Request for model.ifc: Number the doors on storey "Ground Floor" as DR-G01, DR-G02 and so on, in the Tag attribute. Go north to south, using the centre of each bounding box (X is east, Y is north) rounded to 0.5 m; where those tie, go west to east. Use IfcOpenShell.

First a look at what the model holds.

```python
import ifcopenshell
import ifcopenshell.util.element
import ifcopenshell.util.placement

model = ifcopenshell.open("model.ifc")
print(model.schema)
storey = next(s for s in model.by_type("IfcBuildingStorey") if s.Name == "Ground Floor")
doors = [e for e in ifcopenshell.util.element.get_decomposition(storey) if e.is_a("IfcDoor")]
for e in sorted(doors, key=lambda e: e.id()):
    origin = ifcopenshell.util.placement.get_local_placement(e.ObjectPlacement)[:3, 3]
    print(e.id(), e.Tag, e.Name, origin.round(2) + 0.0, sep=" | ")
```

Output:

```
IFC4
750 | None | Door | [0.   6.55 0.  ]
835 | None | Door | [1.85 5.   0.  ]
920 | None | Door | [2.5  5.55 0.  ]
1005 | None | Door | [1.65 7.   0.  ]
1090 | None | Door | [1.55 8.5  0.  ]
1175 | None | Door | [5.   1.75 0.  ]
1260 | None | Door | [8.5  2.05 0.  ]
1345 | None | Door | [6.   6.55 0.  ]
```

```python
import ifcopenshell
import ifcopenshell.geom
import ifcopenshell.util.element
import ifcopenshell.util.shape

model = ifcopenshell.open("model.ifc")
settings = ifcopenshell.geom.settings()
settings.set("use-world-coords", True)


def centre(element):
    shape = ifcopenshell.geom.create_shape(settings, element)
    return ifcopenshell.util.shape.get_bbox_centroid(shape.geometry)


storey = next(s for s in model.by_type("IfcBuildingStorey") if s.Name == "Ground Floor")
doors = [e for e in ifcopenshell.util.element.get_decomposition(storey) if e.is_a("IfcDoor")]

# Insertion points can sit at a corner or the storey origin, so sort by the geometry (in metres).
centres = {e: centre(e) for e in doors}
doors.sort(key=lambda e: (-round(centres[e][1] / 0.5), centres[e][0]))

for i, e in enumerate(doors, start=1):
    number = f"DR-G{i:02d}"
    e.Tag = number
    print(e.id(), number)

model.write("model_edited.ifc")
```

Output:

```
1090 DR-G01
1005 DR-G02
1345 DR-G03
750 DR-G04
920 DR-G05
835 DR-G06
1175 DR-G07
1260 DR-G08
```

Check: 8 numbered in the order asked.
